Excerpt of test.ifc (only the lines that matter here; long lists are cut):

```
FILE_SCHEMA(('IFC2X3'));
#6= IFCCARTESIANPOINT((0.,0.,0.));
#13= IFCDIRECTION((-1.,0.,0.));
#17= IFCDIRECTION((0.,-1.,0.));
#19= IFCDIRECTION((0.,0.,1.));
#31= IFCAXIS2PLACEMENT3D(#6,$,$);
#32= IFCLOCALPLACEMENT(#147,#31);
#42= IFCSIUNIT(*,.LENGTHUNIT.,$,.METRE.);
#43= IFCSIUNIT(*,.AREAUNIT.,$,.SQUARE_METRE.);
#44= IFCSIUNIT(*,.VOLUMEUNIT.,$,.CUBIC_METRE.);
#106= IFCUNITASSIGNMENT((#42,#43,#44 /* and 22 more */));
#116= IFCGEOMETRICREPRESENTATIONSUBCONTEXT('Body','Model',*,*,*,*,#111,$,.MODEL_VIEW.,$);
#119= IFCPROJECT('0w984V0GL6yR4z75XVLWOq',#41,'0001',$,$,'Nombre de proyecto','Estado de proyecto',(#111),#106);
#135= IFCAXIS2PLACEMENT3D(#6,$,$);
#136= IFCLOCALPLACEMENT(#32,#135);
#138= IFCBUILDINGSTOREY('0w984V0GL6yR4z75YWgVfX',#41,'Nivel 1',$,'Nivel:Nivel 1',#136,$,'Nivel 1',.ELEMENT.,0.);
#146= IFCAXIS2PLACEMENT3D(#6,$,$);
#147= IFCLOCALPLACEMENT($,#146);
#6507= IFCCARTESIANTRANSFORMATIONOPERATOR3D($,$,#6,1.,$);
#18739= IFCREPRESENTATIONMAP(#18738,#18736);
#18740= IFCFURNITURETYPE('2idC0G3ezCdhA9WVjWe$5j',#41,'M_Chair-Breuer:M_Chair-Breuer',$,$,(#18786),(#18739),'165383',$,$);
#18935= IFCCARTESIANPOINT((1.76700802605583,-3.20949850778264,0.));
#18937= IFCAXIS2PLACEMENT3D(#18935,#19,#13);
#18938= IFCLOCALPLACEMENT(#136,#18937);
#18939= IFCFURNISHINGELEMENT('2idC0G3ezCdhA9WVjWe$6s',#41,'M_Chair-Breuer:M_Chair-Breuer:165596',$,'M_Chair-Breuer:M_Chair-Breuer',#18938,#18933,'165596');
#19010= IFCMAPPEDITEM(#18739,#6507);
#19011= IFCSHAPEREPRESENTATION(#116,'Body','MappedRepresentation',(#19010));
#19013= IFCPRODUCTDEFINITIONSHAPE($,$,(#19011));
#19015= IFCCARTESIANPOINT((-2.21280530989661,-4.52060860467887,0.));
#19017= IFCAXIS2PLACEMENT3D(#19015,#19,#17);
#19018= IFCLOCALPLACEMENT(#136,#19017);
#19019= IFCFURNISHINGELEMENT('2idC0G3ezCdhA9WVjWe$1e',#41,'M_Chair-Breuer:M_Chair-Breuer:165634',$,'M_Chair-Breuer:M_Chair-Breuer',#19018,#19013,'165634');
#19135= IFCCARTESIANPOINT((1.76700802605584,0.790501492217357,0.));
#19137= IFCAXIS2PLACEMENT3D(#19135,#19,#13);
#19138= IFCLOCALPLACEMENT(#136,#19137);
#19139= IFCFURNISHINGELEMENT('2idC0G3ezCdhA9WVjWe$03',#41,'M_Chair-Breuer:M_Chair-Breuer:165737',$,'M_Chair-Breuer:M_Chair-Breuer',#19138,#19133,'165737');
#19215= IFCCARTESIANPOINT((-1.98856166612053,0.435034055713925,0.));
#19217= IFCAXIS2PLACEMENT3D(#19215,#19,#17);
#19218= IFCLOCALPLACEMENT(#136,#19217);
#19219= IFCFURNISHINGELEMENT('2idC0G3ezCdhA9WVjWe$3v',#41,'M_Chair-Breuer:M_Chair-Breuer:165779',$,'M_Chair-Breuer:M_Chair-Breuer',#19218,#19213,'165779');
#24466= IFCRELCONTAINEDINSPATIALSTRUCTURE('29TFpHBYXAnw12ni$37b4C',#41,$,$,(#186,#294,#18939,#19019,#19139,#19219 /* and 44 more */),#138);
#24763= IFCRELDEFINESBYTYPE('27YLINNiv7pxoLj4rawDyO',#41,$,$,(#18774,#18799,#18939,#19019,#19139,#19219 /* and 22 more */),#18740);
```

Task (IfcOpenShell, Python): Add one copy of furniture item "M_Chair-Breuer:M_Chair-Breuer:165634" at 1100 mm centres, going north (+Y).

```python
import numpy as np
import ifcopenshell
import ifcopenshell.api.geometry
import ifcopenshell.api.root
import ifcopenshell.util.element
import ifcopenshell.util.placement

model = ifcopenshell.open("test.ifc")


def reuse_history(source, copy):
    """copy_class also copies each property set's owner history, people and application; keep the originals."""
    for rel in copy.IsDefinedBy:
        if rel.is_a("IfcRelDefinesByProperties") and (history := rel.RelatingPropertyDefinition.OwnerHistory):
            rel.RelatingPropertyDefinition.OwnerHistory = source.OwnerHistory
            ifcopenshell.util.element.remove_deep2(model, history)


source = model.by_id(19019)
base = ifcopenshell.util.placement.get_local_placement(source.ObjectPlacement)
step = np.array([0.0, 1.0, 0.0]) * 1.1

for i in range(1, 2):
    copy = ifcopenshell.api.root.copy_class(model, product=source)
    copy.Representation = ifcopenshell.util.element.copy_deep(
        model, source.Representation, exclude=["IfcGeometricRepresentationContext", "IfcRepresentationMap"]
    )
    copy.Name = "M_Chair-Breuer:M_Chair-Breuer"
    copy.Tag = None
    reuse_history(source, copy)
    matrix = base.copy()
    matrix[:3, 3] += i * step
    print("added at", matrix[:3, 3].round(3) + 0.0)
    ifcopenshell.api.geometry.edit_object_placement(model, product=copy, matrix=matrix, is_si=False)

model.write("test_edited.ifc")
```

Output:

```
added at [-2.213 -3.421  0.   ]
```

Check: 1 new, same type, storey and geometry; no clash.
